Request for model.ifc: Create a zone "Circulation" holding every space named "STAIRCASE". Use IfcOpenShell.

First a look at what the model holds.

```python
import ifcopenshell

model = ifcopenshell.open("model.ifc")
print(model.schema)
seen = {}
for space in model.by_type("IfcSpace"):
    seen[space.LongName] = seen.get(space.LongName, 0) + 1
for name, count in sorted(seen.items(), key=str):
    print(count, "x", name)
print("zones:", [z.Name for z in model.by_type("IfcZone")][:20])
```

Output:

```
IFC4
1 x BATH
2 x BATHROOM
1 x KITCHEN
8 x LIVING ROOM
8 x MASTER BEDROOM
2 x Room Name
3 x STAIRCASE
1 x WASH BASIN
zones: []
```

```python
import ifcopenshell
import ifcopenshell.api.group
import ifcopenshell.api.root

model = ifcopenshell.open("model.ifc")

names = {"STAIRCASE"}
spaces = [s for s in model.by_type("IfcSpace") if s.LongName in names]

zone = ifcopenshell.api.root.create_entity(model, ifc_class="IfcZone", name="Circulation")
ifcopenshell.api.group.assign_group(model, products=spaces, group=zone)
print(len(spaces), "spaces in", zone.Name)

model.write("model-out.ifc")
```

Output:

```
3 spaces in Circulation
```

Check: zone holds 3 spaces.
